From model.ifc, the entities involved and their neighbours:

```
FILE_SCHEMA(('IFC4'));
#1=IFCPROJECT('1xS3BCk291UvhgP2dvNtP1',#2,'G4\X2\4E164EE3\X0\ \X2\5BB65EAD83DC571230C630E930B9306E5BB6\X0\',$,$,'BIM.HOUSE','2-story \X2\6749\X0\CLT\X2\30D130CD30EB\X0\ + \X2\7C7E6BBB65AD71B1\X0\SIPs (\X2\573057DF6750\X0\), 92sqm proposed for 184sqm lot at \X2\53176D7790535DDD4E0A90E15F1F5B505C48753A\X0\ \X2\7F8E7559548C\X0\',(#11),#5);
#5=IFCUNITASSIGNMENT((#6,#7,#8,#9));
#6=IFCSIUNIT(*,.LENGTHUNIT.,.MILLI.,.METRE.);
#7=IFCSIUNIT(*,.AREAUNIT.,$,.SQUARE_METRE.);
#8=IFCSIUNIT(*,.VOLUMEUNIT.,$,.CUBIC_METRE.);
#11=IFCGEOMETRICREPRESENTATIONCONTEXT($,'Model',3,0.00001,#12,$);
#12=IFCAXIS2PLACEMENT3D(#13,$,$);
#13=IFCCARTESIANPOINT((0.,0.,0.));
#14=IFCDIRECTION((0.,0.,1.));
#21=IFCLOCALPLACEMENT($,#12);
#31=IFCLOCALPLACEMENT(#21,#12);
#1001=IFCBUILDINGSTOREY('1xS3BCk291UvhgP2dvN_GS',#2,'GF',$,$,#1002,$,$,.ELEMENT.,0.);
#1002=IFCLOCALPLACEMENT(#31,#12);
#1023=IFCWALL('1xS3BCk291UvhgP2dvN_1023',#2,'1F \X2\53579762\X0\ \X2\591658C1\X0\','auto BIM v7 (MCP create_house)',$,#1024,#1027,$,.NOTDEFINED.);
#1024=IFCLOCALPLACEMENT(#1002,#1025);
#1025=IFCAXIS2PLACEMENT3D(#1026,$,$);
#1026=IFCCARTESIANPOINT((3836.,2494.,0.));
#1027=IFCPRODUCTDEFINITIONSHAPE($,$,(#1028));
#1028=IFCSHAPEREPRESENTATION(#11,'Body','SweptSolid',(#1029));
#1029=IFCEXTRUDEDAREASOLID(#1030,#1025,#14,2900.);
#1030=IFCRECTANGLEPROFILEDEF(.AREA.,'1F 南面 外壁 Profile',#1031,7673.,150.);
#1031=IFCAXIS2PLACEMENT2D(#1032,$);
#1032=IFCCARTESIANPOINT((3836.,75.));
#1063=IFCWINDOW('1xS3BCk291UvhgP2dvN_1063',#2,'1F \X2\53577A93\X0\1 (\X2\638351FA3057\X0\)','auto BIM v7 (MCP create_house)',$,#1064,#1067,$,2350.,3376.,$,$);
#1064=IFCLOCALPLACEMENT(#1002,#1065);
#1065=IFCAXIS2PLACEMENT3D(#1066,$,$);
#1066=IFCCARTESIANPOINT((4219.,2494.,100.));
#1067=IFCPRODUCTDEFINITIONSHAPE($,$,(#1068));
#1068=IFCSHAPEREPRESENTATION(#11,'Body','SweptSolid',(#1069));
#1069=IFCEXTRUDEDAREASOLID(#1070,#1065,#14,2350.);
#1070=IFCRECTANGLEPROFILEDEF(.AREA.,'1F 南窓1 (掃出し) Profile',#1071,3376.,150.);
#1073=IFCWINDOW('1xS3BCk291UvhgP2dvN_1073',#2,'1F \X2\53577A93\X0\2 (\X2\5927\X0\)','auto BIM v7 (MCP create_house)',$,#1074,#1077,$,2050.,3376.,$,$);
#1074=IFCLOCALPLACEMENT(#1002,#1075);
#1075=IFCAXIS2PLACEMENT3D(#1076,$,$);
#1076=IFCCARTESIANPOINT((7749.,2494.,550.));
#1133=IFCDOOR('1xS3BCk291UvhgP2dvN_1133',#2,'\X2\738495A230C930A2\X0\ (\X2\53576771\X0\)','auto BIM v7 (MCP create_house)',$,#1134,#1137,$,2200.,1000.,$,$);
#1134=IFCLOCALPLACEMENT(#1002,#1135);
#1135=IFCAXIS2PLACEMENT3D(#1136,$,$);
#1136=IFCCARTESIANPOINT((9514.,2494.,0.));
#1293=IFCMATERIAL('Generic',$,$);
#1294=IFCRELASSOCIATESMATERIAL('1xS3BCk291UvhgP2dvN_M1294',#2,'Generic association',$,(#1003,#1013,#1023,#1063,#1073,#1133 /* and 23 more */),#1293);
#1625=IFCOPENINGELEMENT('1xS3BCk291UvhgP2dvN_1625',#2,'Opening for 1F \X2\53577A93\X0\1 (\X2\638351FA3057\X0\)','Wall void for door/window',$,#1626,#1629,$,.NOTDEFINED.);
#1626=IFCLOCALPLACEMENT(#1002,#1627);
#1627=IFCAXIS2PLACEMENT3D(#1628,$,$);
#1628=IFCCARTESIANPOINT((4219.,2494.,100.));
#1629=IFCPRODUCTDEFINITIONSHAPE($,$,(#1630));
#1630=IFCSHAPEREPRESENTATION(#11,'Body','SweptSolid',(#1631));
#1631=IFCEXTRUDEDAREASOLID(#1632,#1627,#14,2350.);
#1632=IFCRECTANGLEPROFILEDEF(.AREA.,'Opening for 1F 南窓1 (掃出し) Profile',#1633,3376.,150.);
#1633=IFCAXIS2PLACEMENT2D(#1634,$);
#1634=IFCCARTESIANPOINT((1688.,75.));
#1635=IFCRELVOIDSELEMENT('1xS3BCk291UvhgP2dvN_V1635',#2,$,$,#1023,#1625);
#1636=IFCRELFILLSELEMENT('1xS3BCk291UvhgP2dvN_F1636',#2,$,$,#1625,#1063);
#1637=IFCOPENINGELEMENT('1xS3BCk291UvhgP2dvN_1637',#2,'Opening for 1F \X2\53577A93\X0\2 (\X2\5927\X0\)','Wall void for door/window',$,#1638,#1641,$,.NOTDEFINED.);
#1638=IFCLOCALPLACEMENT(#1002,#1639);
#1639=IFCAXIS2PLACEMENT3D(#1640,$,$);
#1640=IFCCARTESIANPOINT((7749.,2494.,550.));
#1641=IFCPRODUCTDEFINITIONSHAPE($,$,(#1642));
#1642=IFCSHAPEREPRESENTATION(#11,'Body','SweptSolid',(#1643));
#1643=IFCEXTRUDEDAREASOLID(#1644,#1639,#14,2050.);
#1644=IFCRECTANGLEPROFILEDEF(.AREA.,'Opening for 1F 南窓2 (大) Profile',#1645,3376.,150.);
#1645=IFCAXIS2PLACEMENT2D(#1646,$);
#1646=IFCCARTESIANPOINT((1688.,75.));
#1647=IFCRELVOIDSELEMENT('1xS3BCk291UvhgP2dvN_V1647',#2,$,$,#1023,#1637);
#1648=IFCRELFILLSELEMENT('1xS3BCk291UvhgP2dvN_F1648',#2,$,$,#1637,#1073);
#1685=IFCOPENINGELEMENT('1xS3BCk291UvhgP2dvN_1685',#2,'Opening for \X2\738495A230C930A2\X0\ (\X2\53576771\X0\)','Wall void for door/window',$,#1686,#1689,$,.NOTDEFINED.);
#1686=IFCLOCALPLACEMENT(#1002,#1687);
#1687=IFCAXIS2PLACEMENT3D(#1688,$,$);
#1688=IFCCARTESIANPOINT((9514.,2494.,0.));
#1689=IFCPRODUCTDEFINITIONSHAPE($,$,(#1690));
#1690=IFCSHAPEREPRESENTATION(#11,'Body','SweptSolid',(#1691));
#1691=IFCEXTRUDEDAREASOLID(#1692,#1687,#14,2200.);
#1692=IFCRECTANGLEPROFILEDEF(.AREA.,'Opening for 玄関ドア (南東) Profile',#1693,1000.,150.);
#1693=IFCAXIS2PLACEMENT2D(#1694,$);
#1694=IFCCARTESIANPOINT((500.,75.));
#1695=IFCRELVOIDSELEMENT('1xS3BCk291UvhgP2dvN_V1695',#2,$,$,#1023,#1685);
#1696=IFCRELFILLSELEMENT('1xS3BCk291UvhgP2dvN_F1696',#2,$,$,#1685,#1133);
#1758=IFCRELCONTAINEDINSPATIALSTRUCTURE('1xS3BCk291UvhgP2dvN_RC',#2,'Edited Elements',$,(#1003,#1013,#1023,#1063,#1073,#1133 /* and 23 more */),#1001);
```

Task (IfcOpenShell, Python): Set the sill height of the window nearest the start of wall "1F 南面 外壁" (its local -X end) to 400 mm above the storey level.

```python
import numpy as np
import ifcopenshell
import ifcopenshell.api.geometry
import ifcopenshell.geom
import ifcopenshell.util.element
import ifcopenshell.util.placement
import ifcopenshell.util.shape
import ifcopenshell.util.unit

model = ifcopenshell.open("model.ifc")
unit_scale = ifcopenshell.util.unit.calculate_unit_scale(model)

window = model.by_guid("1xS3BCk291UvhgP2dvN_1063")
opening = window.FillsVoids[0].RelatingOpeningElement
storey = ifcopenshell.util.element.get_container(window, ifc_class="IfcBuildingStorey")
level = ifcopenshell.util.placement.get_local_placement(storey.ObjectPlacement)[2, 3]

# The opening's origin need not be at the sill, so measure its lowest point.
shape = ifcopenshell.geom.create_shape(ifcopenshell.geom.settings(), opening)
bottom = ifcopenshell.util.shape.get_shape_bottom_elevation(shape, shape.geometry) / unit_scale
dz = level + 0.4 / unit_scale - bottom

shift = np.array([0.0, 0.0, dz])
# The window is not placed relative to its opening, so move both.
for product in (opening, window):
    matrix = ifcopenshell.util.placement.get_local_placement(product.ObjectPlacement)
    matrix[:3, 3] += shift
    ifcopenshell.api.geometry.edit_object_placement(model, product=product, matrix=matrix, is_si=False)

print(f"moved by {dz * unit_scale:+.3f} m")

model.write("model_rev.ifc")
```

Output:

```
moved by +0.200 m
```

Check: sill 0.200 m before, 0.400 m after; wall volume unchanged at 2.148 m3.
